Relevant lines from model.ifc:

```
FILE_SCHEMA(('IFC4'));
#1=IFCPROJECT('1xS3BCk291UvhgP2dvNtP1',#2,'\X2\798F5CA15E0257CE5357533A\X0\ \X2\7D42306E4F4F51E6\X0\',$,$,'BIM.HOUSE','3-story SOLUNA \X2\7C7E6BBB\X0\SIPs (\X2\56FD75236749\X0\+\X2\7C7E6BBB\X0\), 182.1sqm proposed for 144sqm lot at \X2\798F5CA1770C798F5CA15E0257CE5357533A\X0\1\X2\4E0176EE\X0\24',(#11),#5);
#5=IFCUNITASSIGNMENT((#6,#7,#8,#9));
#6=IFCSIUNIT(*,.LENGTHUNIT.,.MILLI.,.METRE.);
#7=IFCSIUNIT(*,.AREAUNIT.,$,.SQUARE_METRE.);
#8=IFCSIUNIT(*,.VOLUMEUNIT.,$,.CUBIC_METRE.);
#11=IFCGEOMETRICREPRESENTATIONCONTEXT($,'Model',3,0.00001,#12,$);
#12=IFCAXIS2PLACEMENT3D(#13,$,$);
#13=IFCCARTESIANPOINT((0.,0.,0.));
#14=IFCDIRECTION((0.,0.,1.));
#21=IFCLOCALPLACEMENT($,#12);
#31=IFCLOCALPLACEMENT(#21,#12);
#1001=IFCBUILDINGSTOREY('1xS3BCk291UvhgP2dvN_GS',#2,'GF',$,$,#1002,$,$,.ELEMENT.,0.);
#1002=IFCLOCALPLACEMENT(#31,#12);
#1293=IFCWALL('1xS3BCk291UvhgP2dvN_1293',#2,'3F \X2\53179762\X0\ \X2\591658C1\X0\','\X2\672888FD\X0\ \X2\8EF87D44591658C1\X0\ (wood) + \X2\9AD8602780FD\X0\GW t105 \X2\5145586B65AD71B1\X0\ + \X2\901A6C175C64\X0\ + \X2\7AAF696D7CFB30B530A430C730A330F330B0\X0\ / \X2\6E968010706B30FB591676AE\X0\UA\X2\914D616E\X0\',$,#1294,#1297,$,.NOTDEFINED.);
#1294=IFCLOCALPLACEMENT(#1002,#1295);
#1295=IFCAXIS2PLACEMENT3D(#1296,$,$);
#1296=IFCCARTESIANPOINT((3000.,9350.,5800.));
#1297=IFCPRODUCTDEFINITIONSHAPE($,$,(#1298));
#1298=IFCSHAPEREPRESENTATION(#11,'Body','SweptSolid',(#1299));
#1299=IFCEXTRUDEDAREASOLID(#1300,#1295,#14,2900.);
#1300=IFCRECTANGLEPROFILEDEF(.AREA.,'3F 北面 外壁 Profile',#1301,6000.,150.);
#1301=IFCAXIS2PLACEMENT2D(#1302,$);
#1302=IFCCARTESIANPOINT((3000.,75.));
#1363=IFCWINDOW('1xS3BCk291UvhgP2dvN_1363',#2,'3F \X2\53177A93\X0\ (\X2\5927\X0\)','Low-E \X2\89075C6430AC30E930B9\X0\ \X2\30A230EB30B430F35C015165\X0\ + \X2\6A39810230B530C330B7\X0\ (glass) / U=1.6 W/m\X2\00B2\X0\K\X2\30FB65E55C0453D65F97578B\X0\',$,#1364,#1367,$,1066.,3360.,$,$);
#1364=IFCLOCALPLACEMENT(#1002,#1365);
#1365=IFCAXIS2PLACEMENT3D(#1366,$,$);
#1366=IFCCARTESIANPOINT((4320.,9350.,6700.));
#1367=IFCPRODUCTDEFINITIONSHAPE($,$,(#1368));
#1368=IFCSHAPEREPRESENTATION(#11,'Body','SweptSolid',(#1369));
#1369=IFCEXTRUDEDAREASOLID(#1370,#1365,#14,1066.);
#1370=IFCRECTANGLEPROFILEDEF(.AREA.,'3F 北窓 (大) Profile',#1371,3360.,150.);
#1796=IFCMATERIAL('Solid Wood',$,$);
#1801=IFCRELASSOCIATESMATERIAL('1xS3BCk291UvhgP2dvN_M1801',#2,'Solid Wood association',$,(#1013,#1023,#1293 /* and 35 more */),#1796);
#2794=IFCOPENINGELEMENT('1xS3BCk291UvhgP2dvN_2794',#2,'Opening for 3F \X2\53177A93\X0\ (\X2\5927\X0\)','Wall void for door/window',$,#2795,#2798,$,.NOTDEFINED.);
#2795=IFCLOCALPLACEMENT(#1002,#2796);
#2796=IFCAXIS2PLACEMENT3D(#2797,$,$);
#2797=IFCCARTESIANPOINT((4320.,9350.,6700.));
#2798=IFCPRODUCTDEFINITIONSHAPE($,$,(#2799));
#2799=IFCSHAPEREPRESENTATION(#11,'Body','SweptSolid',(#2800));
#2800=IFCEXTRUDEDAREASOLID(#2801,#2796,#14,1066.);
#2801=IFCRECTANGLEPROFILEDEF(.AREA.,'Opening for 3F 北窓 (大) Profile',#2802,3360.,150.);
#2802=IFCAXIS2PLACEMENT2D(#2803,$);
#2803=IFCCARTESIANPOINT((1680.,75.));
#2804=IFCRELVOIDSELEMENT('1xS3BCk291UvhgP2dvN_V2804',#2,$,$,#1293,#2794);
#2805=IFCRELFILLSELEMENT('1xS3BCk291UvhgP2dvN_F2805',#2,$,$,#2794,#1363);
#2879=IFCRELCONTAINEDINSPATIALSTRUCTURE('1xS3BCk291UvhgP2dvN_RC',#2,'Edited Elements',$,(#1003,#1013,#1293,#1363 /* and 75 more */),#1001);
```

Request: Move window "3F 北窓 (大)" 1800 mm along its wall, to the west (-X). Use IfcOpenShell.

```python
import ifcopenshell
import ifcopenshell.api.geometry
import ifcopenshell.util.placement

model = ifcopenshell.open("model.ifc")

window = model.by_guid("1xS3BCk291UvhgP2dvN_1363")
opening = window.FillsVoids[0].RelatingOpeningElement
wall = opening.VoidsElements[0].RelatingBuildingElement

wall_matrix = ifcopenshell.util.placement.get_local_placement(wall.ObjectPlacement)
shift = wall_matrix[:3, 0] * -1800.0
before = ifcopenshell.util.placement.get_local_placement(window.ObjectPlacement)[:3, 3].copy()

# The window is not placed relative to its opening, so move both.
for product in (opening, window):
    matrix = ifcopenshell.util.placement.get_local_placement(product.ObjectPlacement)
    matrix[:3, 3] += shift
    ifcopenshell.api.geometry.edit_object_placement(model, product=product, matrix=matrix, is_si=False)

after = ifcopenshell.util.placement.get_local_placement(window.ObjectPlacement)[:3, 3]
print("window moved by", (after - before).round(3) + 0.0)

model.write("model_edited.ifc")
```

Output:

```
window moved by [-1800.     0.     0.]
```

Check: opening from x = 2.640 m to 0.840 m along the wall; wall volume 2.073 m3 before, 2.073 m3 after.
